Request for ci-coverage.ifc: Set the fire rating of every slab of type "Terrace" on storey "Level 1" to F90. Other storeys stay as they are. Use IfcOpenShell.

First a look at what the model holds.

```python
import ifcopenshell
import ifcopenshell.util.element

model = ifcopenshell.open("ci-coverage.ifc")
print(model.schema)
storey = next(s for s in model.by_type("IfcBuildingStorey") if s.Name == "Level 1")
slabs = [e for e in ifcopenshell.util.element.get_decomposition(storey) if e.is_a("IfcSlab")]
seen = {}
for e in slabs:
    element_type = ifcopenshell.util.element.get_type(e)
    key = (element_type.Name if element_type != e and element_type else None, ifcopenshell.util.element.get_pset(e, "Pset_SlabCommon", "FireRating"))
    seen[key] = seen.get(key, 0) + 1
for (name, value), count in sorted(seen.items(), key=str):
    print(count, "x", name, "|", value)
```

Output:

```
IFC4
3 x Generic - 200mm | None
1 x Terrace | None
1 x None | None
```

```python
import ifcopenshell
import ifcopenshell.api.pset
import ifcopenshell.util.element

model = ifcopenshell.open("ci-coverage.ifc")

storey = next(s for s in model.by_type("IfcBuildingStorey") if s.Name == "Level 1")
slabs = [e for e in ifcopenshell.util.element.get_decomposition(storey) if e.is_a("IfcSlab")]

count = 0
for e in slabs:
    element_type = ifcopenshell.util.element.get_type(e)
    if element_type in (None, e) or element_type.Name != "Terrace":
        continue
    # add_pset returns the element's existing set when there is one.
    pset = ifcopenshell.api.pset.add_pset(model, product=e, name="Pset_SlabCommon")
    ifcopenshell.api.pset.edit_pset(model, pset=pset, properties={"FireRating": "F90"})
    count += 1

print(count, "slabs updated")

model.write("ci-coverage_edited.ifc")
```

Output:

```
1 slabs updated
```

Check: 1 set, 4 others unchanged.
